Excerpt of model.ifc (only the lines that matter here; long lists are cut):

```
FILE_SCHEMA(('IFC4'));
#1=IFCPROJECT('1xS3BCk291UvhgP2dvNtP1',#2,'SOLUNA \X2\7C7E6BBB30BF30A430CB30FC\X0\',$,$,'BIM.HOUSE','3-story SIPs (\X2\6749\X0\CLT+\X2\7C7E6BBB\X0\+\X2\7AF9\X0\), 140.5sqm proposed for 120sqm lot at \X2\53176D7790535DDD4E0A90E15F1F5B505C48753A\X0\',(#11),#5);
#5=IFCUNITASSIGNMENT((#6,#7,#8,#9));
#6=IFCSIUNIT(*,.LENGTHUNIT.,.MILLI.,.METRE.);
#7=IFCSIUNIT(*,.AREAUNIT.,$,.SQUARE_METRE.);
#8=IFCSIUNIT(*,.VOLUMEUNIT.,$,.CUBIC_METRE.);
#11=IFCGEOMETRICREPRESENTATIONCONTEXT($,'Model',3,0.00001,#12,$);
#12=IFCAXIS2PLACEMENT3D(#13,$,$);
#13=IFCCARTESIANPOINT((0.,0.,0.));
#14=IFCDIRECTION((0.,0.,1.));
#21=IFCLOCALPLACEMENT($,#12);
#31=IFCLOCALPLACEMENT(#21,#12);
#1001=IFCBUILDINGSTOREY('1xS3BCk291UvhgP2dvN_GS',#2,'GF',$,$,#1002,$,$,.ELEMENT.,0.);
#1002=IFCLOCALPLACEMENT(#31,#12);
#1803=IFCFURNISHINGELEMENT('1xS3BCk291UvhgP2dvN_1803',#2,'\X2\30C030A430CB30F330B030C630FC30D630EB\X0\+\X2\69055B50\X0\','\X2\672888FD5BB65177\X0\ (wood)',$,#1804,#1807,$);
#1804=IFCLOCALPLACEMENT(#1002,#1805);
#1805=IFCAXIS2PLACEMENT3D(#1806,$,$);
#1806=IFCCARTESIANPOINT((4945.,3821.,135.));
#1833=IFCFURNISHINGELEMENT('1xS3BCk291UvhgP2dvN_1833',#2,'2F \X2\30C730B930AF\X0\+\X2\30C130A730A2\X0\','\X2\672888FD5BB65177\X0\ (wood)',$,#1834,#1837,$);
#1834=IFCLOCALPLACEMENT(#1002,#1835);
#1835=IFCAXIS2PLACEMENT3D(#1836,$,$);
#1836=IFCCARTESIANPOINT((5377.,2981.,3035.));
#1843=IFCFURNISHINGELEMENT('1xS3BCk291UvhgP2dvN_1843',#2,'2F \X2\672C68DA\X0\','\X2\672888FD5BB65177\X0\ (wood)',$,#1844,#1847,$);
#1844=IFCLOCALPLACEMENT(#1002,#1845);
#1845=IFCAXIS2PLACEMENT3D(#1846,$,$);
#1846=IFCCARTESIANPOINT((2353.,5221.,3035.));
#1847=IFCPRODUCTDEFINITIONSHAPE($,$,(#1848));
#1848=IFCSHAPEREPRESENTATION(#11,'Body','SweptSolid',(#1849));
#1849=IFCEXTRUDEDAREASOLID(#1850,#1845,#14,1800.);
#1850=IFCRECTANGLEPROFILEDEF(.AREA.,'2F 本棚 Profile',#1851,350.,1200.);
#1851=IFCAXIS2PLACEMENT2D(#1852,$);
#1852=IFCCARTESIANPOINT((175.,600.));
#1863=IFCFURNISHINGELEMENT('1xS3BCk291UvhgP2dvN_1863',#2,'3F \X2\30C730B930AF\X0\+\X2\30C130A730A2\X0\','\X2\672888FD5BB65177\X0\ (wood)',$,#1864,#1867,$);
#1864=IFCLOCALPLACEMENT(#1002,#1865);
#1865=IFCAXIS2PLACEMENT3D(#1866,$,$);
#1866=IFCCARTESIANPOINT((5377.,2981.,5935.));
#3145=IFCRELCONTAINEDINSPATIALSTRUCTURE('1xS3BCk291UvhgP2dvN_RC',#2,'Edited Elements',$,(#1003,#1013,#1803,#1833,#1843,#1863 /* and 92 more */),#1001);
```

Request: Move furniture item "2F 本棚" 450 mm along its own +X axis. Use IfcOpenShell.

```python
import ifcopenshell
import ifcopenshell.api.geometry
import ifcopenshell.util.placement

model = ifcopenshell.open("model.ifc")

item = model.by_guid("1xS3BCk291UvhgP2dvN_1843")
matrix = ifcopenshell.util.placement.get_local_placement(item.ObjectPlacement)
matrix[:3, 3] += matrix[:3, 0] * 450.0
ifcopenshell.api.geometry.edit_object_placement(model, product=item, matrix=matrix, is_si=False)

print(ifcopenshell.util.placement.get_local_placement(item.ObjectPlacement).round(3) + 0.0)

model.write("model-out.ifc")
```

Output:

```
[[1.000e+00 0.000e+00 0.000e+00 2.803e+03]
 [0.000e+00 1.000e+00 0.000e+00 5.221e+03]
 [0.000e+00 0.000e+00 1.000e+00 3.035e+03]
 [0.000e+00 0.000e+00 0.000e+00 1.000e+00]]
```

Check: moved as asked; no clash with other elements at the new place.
